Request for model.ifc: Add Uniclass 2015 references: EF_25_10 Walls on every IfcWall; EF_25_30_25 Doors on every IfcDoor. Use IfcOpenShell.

First a look at what the model holds.

```python
import ifcopenshell

model = ifcopenshell.open("model.ifc")
print(model.schema)
print("classifications:", [c.Name for c in model.by_type("IfcClassification")])
for ifc_class in ("IfcDoor", "IfcRoof", "IfcStair", "IfcWall", "IfcWindow"):
    print(ifc_class, len(model.by_type(ifc_class)))
```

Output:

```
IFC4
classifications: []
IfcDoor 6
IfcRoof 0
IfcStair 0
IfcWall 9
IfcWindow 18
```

```python
import ifcopenshell
import ifcopenshell.api.classification

model = ifcopenshell.open("model.ifc")

system = ifcopenshell.api.classification.add_classification(model, classification="Uniclass 2015")

codes = {
    "IfcWall": ("EF_25_10", "Walls"),
    "IfcDoor": ("EF_25_30_25", "Doors"),
}
for ifc_class, (code, name) in codes.items():
    products = model.by_type(ifc_class)
    ifcopenshell.api.classification.add_reference(
        model, products=products, classification=system, identification=code, name=name
    )
    print(code, len(products))

model.write("model-out.ifc")
```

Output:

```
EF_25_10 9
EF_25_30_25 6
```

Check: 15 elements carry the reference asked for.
